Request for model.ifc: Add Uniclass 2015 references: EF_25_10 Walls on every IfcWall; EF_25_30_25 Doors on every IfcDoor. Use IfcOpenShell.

First a look at what the model holds.

```python
import ifcopenshell

model = ifcopenshell.open("model.ifc")
print(model.schema)
print("classifications:", [c.Name for c in model.by_type("IfcClassification")])
for ifc_class in ("IfcDoor", "IfcRoof", "IfcStair", "IfcWall", "IfcWindow"):
    print(ifc_class, len(model.by_type(ifc_class)))
```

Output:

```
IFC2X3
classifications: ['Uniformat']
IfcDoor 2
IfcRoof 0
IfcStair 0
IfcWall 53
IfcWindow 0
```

```python
import ifcopenshell
import ifcopenshell.api.classification

model = ifcopenshell.open("model.ifc")

# IFC2X3 requires Source and Edition and has no link from the project to the system.
system = model.create_entity("IfcClassification", Source="NBS", Edition="2015", Name="Uniclass 2015")

codes = {
    "IfcWall": ("EF_25_10", "Walls"),
    "IfcDoor": ("EF_25_30_25", "Doors"),
}
for ifc_class, (code, name) in codes.items():
    products = model.by_type(ifc_class)
    ifcopenshell.api.classification.add_reference(
        model, products=products, classification=system, identification=code, name=name
    )
    print(code, len(products))

model.write("model_rev.ifc")
```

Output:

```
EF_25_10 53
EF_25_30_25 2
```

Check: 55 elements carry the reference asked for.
